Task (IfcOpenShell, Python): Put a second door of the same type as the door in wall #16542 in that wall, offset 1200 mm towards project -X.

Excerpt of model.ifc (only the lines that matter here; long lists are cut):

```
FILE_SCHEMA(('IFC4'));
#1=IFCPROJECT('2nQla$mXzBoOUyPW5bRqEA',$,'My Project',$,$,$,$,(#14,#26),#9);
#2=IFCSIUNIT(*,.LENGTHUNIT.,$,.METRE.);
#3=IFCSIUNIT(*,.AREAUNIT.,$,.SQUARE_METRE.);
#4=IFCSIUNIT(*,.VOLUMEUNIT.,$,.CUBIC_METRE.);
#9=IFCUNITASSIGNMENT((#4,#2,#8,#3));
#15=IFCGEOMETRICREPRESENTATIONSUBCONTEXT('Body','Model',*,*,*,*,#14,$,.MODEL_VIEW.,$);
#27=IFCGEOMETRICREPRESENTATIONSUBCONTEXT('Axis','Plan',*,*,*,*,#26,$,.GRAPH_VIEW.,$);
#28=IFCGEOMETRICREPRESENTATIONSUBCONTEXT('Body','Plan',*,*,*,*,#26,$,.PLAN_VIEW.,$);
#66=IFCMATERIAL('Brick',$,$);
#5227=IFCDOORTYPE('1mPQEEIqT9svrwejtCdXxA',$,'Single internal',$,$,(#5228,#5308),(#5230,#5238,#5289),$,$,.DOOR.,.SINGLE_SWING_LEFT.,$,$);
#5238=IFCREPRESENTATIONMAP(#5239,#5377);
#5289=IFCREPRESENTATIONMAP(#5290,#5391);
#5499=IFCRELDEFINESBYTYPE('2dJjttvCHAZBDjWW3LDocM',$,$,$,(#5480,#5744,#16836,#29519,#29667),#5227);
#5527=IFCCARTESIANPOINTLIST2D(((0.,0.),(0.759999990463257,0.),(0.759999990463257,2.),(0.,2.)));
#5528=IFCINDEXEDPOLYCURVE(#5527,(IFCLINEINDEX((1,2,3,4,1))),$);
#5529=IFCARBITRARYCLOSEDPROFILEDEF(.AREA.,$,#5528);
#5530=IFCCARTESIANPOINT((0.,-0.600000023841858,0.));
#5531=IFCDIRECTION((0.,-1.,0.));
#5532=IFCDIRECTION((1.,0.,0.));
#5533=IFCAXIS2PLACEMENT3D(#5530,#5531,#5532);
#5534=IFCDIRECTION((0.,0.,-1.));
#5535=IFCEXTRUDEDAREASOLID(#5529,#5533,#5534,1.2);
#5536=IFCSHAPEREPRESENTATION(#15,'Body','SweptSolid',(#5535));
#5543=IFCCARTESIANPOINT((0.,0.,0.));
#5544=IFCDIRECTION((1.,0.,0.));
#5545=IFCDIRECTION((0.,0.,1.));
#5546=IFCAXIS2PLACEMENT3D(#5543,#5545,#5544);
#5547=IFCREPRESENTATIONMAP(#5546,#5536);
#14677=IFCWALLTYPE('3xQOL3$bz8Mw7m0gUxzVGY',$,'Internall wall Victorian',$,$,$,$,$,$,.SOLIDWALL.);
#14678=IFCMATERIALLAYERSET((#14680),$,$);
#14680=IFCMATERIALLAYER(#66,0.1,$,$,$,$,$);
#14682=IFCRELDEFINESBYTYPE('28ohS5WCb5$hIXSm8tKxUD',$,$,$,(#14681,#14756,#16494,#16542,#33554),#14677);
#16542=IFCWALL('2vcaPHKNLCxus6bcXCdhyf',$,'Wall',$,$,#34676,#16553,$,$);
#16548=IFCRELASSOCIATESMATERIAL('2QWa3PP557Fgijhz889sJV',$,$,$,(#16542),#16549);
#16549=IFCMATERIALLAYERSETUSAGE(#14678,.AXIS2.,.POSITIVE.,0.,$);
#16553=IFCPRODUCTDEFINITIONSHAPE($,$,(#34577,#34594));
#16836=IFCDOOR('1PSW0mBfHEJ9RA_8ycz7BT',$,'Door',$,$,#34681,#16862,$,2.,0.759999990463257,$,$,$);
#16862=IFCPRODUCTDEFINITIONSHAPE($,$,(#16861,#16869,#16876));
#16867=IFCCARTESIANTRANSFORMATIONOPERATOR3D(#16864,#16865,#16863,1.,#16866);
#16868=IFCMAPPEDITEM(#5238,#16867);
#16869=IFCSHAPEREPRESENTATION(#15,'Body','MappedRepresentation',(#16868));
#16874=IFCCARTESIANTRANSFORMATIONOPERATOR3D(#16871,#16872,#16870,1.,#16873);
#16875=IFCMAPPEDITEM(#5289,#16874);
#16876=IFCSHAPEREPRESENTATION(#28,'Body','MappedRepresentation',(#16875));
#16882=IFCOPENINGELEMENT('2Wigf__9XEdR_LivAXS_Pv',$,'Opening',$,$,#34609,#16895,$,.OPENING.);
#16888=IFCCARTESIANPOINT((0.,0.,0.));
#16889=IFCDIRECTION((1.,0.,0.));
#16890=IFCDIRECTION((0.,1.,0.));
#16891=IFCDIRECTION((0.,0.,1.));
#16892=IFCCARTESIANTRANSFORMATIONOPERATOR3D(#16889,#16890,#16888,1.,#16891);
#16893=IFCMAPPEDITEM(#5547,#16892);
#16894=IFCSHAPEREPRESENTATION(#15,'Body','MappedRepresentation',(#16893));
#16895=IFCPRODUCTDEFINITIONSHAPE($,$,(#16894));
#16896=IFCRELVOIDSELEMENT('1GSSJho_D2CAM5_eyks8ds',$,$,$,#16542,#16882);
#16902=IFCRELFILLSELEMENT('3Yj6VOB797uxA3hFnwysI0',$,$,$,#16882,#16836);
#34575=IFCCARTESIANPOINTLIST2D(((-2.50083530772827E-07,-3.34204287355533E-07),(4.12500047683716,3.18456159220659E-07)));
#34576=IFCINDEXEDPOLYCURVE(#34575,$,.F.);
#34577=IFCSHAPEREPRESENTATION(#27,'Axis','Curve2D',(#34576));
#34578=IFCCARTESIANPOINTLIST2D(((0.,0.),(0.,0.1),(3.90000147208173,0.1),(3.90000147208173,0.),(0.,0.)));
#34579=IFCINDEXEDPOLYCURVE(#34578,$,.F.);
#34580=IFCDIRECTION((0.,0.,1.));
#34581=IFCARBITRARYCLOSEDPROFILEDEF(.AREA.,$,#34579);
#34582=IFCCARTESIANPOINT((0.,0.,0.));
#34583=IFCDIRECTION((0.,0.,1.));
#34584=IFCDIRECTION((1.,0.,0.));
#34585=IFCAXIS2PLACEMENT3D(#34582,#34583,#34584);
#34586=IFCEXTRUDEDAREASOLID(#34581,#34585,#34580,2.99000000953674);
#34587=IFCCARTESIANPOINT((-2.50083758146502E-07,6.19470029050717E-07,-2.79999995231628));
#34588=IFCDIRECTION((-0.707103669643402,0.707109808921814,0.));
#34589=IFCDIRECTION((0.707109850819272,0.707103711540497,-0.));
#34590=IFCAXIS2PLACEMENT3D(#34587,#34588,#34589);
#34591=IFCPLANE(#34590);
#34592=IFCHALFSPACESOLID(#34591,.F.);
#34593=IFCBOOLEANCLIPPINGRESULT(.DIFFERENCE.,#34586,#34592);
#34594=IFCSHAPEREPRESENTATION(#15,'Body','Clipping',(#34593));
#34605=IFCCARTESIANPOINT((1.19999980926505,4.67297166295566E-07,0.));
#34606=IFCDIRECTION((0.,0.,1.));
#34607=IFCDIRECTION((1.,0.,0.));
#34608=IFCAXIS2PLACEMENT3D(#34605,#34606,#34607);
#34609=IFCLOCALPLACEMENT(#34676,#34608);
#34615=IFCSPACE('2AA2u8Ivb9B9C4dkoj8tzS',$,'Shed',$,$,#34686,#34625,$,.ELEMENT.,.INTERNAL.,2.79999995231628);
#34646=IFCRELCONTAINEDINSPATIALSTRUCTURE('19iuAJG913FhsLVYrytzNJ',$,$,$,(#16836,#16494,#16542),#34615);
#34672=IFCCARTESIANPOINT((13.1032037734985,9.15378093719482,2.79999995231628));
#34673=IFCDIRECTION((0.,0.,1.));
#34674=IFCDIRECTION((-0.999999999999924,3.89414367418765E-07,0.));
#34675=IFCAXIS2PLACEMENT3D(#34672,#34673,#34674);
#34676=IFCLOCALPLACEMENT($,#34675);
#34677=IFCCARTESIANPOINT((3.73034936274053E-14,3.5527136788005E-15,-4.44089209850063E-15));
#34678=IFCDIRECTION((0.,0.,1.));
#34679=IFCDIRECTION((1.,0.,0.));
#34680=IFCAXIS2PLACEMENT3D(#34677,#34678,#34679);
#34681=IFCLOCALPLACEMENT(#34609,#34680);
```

```python
import ifcopenshell
import ifcopenshell.api.feature
import ifcopenshell.api.geometry
import ifcopenshell.api.root
import ifcopenshell.geom
import ifcopenshell.util.element
import ifcopenshell.util.placement
import ifcopenshell.util.shape

model = ifcopenshell.open("model.ifc")
settings = ifcopenshell.geom.settings()


def volume(element):
    """Net volume in cubic metres, openings subtracted."""
    shape = ifcopenshell.geom.create_shape(settings, element)
    return ifcopenshell.util.shape.get_volume(shape.geometry)


door = model.by_id(16836)
opening = door.FillsVoids[0].RelatingOpeningElement
wall = opening.VoidsElements[0].RelatingBuildingElement
before = volume(wall)
shift = ifcopenshell.util.placement.get_local_placement(wall.ObjectPlacement)[:3, 0] * 1.2

# copy_class copies the void relationship, type, container and properties, but no geometry.
new_opening = ifcopenshell.api.root.copy_class(model, product=opening)
new_opening.Representation = ifcopenshell.util.element.copy_deep(
    model, opening.Representation, exclude=["IfcGeometricRepresentationContext", "IfcRepresentationMap"]
)
new_door = ifcopenshell.api.root.copy_class(model, product=door)
new_door.Representation = ifcopenshell.util.element.copy_deep(
    model, door.Representation, exclude=["IfcGeometricRepresentationContext", "IfcRepresentationMap"]
)
ifcopenshell.api.feature.add_filling(model, opening=new_opening, element=new_door)

for old, new in ((opening, new_opening), (door, new_door)):
    matrix = ifcopenshell.util.placement.get_local_placement(old.ObjectPlacement)
    matrix[:3, 3] += shift
    ifcopenshell.api.geometry.edit_object_placement(model, product=new, matrix=matrix, is_si=False)

after = volume(wall)

print(f"wall volume {before:.3f} -> {after:.3f} m3")

model.write("model_edited.ifc")
```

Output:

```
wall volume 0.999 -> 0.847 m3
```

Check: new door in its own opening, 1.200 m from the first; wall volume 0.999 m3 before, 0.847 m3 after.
